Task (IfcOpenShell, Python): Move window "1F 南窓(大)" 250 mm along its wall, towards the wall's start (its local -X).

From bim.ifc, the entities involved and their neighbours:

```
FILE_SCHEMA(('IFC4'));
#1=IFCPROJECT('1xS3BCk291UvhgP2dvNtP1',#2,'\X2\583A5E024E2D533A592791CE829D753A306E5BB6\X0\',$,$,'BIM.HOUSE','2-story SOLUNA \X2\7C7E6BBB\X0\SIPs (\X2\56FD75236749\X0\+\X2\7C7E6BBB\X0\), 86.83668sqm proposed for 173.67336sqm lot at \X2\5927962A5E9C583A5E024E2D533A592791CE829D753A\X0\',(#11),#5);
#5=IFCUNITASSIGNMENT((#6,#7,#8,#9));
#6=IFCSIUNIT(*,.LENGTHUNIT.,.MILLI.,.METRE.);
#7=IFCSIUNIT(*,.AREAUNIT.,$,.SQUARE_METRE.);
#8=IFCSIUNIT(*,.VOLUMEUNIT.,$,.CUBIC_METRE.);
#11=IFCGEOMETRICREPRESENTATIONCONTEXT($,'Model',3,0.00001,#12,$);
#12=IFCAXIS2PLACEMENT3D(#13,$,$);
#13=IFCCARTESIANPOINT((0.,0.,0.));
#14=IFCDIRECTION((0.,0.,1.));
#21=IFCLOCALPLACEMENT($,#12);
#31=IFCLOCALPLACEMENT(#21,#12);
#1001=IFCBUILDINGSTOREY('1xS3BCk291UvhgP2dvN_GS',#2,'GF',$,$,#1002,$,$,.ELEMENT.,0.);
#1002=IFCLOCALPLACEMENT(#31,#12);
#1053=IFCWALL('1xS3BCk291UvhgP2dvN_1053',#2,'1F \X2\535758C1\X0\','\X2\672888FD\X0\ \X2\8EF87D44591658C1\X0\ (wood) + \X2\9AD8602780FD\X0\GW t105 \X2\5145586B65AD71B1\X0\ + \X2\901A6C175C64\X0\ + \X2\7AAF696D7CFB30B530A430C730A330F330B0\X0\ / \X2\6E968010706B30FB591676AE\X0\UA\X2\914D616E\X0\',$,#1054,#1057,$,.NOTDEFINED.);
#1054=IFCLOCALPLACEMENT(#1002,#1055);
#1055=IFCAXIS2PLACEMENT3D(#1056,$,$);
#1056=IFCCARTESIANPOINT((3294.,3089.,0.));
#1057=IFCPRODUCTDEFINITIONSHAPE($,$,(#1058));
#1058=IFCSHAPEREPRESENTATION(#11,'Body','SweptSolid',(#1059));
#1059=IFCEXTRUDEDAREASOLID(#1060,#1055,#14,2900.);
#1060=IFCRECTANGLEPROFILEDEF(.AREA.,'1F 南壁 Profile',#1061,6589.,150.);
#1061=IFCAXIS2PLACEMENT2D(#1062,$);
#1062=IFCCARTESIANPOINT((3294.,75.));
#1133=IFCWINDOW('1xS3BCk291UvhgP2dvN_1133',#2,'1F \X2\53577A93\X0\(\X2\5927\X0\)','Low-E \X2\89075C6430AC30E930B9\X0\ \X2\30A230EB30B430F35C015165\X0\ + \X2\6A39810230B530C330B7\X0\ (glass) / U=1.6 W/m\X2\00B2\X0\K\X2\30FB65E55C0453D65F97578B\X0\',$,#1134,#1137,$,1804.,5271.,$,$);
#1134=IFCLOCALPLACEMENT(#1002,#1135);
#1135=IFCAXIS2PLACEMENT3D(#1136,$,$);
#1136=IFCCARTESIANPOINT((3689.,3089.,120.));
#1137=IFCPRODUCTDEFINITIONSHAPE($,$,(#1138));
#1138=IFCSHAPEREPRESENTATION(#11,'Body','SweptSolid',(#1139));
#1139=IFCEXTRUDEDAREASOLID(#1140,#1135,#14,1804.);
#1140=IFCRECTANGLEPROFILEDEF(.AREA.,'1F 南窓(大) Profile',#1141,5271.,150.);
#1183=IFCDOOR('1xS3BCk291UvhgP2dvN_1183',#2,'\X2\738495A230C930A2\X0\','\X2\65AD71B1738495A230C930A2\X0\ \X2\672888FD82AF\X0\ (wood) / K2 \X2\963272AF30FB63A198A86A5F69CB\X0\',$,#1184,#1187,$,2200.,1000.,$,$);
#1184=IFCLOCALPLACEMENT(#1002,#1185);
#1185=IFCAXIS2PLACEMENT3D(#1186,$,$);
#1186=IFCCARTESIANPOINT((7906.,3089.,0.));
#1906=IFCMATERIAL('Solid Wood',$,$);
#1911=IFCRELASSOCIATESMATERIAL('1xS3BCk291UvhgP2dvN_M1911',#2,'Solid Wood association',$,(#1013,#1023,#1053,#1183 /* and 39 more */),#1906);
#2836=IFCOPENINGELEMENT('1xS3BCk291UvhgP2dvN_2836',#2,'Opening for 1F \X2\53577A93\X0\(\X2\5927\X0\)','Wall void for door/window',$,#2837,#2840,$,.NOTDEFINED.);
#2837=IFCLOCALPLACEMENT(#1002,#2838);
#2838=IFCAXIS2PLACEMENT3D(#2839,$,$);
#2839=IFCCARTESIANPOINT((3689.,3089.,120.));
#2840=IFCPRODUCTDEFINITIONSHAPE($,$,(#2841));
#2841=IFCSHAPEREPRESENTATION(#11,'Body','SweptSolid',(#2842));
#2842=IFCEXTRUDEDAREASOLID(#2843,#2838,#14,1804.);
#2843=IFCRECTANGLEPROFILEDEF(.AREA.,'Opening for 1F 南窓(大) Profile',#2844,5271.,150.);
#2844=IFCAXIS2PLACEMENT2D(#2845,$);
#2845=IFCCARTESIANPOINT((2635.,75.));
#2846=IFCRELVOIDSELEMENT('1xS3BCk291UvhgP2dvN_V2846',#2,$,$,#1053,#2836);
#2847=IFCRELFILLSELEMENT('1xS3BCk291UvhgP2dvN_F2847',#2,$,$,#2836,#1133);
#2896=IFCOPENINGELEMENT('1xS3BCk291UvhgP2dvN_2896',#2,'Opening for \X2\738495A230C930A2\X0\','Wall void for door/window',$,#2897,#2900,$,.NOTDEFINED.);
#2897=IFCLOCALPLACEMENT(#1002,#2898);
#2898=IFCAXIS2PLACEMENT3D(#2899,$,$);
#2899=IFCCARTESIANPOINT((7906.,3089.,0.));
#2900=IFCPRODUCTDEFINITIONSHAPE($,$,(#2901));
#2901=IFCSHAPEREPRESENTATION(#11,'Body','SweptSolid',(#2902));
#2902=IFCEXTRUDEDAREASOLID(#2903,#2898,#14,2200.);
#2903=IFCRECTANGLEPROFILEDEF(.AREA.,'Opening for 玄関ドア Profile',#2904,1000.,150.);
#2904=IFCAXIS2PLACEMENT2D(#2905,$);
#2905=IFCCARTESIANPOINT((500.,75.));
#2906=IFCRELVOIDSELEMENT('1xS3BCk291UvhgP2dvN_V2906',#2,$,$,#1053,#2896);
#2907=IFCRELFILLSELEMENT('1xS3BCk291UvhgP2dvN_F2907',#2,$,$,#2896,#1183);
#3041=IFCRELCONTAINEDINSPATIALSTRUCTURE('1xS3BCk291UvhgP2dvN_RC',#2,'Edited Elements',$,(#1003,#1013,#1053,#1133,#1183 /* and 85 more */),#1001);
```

```python
import ifcopenshell
import ifcopenshell.api.geometry
import ifcopenshell.util.placement

model = ifcopenshell.open("bim.ifc")

window = model.by_guid("1xS3BCk291UvhgP2dvN_1133")
opening = window.FillsVoids[0].RelatingOpeningElement
wall = opening.VoidsElements[0].RelatingBuildingElement

wall_matrix = ifcopenshell.util.placement.get_local_placement(wall.ObjectPlacement)
shift = wall_matrix[:3, 0] * -250.0
before = ifcopenshell.util.placement.get_local_placement(window.ObjectPlacement)[:3, 3].copy()

# The window is not placed relative to its opening, so move both.
for product in (opening, window):
    matrix = ifcopenshell.util.placement.get_local_placement(product.ObjectPlacement)
    matrix[:3, 3] += shift
    ifcopenshell.api.geometry.edit_object_placement(model, product=product, matrix=matrix, is_si=False)

after = ifcopenshell.util.placement.get_local_placement(window.ObjectPlacement)[:3, 3]
print("window moved by", (after - before).round(3) + 0.0)

model.write("bim_edited.ifc")
```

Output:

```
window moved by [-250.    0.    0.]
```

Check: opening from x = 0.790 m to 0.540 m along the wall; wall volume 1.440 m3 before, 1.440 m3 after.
